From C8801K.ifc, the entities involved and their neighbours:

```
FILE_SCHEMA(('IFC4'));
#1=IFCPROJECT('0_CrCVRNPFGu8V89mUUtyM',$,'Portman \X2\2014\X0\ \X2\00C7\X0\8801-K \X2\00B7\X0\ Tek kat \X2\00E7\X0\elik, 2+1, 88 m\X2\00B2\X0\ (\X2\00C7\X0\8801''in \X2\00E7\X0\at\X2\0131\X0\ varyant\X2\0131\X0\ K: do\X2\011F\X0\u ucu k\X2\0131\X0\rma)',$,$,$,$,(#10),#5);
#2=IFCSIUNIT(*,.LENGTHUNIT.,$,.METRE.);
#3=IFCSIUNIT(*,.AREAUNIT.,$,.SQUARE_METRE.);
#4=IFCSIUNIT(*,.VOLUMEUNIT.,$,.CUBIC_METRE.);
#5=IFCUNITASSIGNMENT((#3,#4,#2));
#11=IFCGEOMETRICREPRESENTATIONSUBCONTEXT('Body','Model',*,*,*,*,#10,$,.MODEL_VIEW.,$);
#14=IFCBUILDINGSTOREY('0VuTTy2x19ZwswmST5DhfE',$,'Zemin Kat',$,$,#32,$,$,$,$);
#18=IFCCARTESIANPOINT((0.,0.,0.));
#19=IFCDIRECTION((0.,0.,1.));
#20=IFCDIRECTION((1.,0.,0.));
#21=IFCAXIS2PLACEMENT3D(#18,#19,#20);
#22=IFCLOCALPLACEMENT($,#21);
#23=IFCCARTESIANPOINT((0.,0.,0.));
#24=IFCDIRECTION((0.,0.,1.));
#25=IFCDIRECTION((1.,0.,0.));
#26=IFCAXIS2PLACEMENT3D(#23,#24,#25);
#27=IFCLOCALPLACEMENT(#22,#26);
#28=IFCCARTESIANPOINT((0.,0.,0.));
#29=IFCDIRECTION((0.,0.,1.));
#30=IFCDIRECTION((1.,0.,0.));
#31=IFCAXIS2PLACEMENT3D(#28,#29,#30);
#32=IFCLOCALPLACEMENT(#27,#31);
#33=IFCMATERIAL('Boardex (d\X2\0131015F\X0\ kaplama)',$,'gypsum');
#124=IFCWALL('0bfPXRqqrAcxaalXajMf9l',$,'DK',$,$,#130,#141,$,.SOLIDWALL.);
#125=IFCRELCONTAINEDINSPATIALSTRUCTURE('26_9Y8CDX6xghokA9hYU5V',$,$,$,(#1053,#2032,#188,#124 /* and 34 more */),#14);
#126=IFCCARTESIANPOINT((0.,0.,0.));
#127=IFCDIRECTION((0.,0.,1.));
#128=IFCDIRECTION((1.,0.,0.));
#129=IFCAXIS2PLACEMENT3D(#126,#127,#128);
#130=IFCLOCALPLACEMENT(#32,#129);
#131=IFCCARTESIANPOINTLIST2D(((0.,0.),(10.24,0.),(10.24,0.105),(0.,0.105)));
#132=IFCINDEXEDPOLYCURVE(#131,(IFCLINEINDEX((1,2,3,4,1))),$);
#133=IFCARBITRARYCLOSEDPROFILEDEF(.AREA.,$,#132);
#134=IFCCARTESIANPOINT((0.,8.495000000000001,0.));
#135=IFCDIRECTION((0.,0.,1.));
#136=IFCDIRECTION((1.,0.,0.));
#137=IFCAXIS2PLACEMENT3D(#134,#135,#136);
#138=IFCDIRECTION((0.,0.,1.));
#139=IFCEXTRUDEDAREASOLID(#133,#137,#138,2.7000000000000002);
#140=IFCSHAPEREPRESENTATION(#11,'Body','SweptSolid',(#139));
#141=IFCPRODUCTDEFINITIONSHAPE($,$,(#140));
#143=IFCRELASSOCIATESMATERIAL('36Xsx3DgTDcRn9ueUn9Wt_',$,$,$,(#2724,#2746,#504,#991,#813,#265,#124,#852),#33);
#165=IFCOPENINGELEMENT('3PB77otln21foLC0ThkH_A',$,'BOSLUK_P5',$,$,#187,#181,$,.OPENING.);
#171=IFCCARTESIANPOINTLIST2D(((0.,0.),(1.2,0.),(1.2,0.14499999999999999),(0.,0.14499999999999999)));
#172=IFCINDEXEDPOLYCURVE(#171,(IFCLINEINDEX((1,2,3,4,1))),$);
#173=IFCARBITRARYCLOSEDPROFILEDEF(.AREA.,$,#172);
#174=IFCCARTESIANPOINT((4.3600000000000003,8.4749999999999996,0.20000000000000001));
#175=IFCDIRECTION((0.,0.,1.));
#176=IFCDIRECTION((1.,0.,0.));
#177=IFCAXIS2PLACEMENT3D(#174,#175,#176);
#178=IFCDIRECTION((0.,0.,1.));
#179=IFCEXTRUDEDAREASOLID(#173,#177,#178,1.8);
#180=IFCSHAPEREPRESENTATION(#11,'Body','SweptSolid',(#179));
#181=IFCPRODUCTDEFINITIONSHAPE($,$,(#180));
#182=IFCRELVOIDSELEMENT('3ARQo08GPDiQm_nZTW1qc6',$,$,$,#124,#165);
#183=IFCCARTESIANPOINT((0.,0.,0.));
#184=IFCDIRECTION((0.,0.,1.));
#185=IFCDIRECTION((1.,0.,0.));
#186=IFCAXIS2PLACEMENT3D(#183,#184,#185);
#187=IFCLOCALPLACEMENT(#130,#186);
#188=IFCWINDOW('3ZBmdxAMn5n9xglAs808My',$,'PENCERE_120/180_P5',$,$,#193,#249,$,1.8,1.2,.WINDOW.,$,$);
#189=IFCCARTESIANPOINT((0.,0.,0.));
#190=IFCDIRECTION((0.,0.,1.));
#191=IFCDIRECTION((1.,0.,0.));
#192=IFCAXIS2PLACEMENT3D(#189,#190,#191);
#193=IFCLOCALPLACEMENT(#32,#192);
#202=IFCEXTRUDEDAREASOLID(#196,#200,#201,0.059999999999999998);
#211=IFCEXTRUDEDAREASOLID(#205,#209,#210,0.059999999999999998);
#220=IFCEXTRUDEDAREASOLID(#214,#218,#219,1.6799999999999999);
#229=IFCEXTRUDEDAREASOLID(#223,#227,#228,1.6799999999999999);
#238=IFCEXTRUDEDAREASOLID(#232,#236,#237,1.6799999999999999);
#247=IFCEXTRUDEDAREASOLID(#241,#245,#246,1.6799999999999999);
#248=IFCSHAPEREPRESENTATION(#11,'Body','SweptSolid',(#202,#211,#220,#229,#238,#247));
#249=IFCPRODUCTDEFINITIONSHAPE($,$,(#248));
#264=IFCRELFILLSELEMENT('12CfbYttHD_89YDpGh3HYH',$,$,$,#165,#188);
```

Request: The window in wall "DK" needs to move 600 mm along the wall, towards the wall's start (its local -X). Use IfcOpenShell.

```python
import ifcopenshell
import ifcopenshell.api.geometry
import ifcopenshell.util.placement
import ifcopenshell.util.unit

model = ifcopenshell.open("C8801K.ifc")
unit_scale = ifcopenshell.util.unit.calculate_unit_scale(model)

window = model.by_guid("3ZBmdxAMn5n9xglAs808My")
opening = window.FillsVoids[0].RelatingOpeningElement
wall = opening.VoidsElements[0].RelatingBuildingElement

wall_matrix = ifcopenshell.util.placement.get_local_placement(wall.ObjectPlacement)
shift = wall_matrix[:3, 0] * -0.6 / unit_scale
before = ifcopenshell.util.placement.get_local_placement(window.ObjectPlacement)[:3, 3].copy()

# The window is not placed relative to its opening, so move both.
for product in (opening, window):
    matrix = ifcopenshell.util.placement.get_local_placement(product.ObjectPlacement)
    matrix[:3, 3] += shift
    ifcopenshell.api.geometry.edit_object_placement(model, product=product, matrix=matrix, is_si=False)

after = ifcopenshell.util.placement.get_local_placement(window.ObjectPlacement)[:3, 3]
print("window moved by", (after - before).round(3) + 0.0)

model.write("C8801K_v2.ifc")
```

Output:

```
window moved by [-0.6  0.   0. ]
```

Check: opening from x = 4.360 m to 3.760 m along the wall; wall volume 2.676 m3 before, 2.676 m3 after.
